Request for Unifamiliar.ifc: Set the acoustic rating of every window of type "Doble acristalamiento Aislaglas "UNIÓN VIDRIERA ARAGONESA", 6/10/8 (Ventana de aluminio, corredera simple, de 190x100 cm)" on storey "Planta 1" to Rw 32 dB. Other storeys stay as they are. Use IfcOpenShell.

First a look at what the model holds.

```python
import ifcopenshell
import ifcopenshell.util.element

model = ifcopenshell.open("Unifamiliar.ifc")
print(model.schema)
storey = next(s for s in model.by_type("IfcBuildingStorey") if s.Name == "Planta 1")
windows = [e for e in ifcopenshell.util.element.get_decomposition(storey) if e.is_a("IfcWindow")]
seen = {}
for e in windows:
    element_type = ifcopenshell.util.element.get_type(e)
    key = (element_type.Name if element_type != e and element_type else None, ifcopenshell.util.element.get_pset(e, "Pset_WindowCommon", "AcousticRating"))
    seen[key] = seen.get(key, 0) + 1
for (name, value), count in sorted(seen.items(), key=str):
    print(count, "x", name, "|", value)
```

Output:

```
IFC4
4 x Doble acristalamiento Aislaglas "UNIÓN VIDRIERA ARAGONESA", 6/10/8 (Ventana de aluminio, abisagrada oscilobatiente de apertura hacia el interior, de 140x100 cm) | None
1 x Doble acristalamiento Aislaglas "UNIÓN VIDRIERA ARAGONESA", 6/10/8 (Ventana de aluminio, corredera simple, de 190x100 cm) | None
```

```python
import ifcopenshell
import ifcopenshell.api.pset
import ifcopenshell.util.element

model = ifcopenshell.open("Unifamiliar.ifc")

storey = next(s for s in model.by_type("IfcBuildingStorey") if s.Name == "Planta 1")
windows = [e for e in ifcopenshell.util.element.get_decomposition(storey) if e.is_a("IfcWindow")]

count = 0
for e in windows:
    element_type = ifcopenshell.util.element.get_type(e)
    if element_type in (None, e) or element_type.Name != 'Doble acristalamiento Aislaglas "UNIÓN VIDRIERA ARAGONESA", 6/10/8 (Ventana de aluminio, corredera simple, de 190x100 cm)':
        continue
    # add_pset returns the element's existing set when there is one.
    pset = ifcopenshell.api.pset.add_pset(model, product=e, name="Pset_WindowCommon")
    ifcopenshell.api.pset.edit_pset(model, pset=pset, properties={"AcousticRating": "Rw 32 dB"})
    count += 1

print(count, "windows updated")

model.write("Unifamiliar_v2.ifc")
```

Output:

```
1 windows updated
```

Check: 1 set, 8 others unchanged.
